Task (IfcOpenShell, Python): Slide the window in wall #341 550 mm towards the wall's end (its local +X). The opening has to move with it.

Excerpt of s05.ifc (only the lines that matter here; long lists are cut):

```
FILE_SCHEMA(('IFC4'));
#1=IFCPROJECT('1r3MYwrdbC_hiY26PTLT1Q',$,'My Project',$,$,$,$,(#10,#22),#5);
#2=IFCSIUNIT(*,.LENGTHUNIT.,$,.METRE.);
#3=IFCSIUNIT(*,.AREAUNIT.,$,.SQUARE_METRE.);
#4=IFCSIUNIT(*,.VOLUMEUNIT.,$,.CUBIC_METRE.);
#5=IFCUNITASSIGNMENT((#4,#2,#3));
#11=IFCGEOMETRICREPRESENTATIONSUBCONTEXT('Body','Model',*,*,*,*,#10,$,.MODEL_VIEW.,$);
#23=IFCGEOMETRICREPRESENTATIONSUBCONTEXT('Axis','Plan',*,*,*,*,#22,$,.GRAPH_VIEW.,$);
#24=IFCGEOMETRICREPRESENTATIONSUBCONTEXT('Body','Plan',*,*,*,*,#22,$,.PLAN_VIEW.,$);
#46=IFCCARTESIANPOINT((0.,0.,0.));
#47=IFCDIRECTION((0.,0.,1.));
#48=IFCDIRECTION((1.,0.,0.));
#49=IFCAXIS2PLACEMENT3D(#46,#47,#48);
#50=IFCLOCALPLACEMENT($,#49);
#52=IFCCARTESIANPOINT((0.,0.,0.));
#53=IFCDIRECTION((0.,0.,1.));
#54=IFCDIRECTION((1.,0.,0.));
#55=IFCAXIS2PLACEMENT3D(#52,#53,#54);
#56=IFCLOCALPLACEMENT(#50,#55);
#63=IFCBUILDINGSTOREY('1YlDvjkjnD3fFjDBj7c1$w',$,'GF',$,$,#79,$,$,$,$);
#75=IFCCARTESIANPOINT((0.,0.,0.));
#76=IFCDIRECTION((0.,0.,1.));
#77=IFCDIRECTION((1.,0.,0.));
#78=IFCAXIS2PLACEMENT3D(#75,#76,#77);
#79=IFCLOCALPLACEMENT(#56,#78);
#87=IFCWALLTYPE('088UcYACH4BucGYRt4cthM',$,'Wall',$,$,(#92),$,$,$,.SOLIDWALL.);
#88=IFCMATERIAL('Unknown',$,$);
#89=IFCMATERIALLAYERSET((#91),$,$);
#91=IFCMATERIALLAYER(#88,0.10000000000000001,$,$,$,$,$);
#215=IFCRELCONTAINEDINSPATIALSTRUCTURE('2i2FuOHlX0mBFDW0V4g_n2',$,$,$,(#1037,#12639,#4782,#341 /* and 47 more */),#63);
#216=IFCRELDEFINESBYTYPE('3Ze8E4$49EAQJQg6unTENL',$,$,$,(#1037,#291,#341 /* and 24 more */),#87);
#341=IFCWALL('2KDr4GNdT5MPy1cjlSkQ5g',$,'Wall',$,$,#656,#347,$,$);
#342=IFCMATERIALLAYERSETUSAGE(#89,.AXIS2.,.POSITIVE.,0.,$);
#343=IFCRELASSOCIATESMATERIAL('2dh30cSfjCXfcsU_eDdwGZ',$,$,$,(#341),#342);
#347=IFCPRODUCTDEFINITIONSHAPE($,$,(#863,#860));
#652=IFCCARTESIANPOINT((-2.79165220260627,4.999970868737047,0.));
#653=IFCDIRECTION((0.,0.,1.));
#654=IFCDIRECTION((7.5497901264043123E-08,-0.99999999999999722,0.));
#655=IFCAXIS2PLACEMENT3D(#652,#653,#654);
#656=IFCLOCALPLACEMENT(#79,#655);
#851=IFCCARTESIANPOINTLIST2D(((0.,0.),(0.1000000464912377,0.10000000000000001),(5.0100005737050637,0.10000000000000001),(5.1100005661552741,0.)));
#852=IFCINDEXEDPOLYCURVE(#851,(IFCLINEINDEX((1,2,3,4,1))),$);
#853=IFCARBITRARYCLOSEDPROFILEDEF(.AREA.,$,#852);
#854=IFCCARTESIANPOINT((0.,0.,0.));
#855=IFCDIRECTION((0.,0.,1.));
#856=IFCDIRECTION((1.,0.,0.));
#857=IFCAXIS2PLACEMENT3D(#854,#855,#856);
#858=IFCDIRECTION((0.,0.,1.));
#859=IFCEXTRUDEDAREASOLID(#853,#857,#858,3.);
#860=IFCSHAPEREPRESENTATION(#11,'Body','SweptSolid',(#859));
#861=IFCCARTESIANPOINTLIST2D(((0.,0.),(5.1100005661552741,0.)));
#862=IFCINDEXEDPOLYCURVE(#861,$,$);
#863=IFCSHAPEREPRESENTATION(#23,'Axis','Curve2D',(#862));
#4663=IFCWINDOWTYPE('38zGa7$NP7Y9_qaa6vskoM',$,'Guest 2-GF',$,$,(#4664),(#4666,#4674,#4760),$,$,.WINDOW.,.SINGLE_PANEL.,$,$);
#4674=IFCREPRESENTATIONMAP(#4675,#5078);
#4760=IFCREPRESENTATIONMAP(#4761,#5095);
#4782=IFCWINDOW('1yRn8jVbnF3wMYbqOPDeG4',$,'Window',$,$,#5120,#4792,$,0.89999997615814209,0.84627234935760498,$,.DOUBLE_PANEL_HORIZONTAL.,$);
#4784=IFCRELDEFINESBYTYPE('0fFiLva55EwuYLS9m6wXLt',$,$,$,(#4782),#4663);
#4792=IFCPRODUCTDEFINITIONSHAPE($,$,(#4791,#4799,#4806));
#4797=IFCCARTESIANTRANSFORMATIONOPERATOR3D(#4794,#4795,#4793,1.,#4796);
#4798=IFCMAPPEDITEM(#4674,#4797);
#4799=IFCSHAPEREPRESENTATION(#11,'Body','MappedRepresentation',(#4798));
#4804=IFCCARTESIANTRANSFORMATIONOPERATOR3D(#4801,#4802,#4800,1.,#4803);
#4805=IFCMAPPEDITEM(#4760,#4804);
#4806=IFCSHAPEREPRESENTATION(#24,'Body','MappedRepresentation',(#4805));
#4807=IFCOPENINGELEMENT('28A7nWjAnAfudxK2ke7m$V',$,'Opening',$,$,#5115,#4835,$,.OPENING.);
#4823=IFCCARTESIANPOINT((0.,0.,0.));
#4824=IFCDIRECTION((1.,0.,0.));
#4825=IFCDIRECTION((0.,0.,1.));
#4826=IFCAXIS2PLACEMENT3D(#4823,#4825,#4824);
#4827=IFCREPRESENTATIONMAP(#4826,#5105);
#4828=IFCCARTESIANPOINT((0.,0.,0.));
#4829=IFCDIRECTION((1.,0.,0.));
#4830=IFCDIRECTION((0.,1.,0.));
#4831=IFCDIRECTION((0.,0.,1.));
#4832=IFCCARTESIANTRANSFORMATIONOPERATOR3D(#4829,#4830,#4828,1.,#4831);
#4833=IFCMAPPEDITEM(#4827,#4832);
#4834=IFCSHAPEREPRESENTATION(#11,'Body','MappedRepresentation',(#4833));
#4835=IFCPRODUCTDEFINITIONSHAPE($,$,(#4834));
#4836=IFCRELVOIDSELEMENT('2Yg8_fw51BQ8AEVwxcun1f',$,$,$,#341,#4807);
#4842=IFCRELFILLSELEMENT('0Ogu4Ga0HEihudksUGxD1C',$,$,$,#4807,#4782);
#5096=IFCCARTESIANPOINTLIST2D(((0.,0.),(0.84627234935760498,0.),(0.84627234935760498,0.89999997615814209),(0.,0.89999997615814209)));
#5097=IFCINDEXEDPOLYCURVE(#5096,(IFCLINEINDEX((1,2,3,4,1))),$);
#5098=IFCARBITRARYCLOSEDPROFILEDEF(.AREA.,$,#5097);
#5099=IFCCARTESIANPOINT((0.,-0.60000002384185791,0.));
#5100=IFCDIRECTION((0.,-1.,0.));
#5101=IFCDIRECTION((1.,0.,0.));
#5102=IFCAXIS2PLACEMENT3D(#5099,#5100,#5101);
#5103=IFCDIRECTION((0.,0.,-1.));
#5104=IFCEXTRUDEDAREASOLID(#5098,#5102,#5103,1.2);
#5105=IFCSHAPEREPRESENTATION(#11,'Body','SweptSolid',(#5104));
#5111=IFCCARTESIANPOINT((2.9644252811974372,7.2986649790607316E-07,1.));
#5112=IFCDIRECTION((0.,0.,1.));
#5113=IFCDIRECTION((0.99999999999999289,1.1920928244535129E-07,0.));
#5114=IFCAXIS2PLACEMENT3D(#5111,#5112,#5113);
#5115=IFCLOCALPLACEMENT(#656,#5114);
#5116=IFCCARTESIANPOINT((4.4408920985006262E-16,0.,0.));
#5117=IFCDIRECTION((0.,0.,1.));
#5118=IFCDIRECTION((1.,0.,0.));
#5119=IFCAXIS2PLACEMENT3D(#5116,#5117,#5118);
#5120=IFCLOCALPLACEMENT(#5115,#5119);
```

```python
import ifcopenshell
import ifcopenshell.api.geometry
import ifcopenshell.util.placement

model = ifcopenshell.open("s05.ifc")

window = model.by_id(4782)
opening = window.FillsVoids[0].RelatingOpeningElement
wall = opening.VoidsElements[0].RelatingBuildingElement

wall_matrix = ifcopenshell.util.placement.get_local_placement(wall.ObjectPlacement)
shift = wall_matrix[:3, 0] * 0.55
before = ifcopenshell.util.placement.get_local_placement(window.ObjectPlacement)[:3, 3].copy()

# The window is placed relative to its opening, so it follows when the opening moves.
matrix = ifcopenshell.util.placement.get_local_placement(opening.ObjectPlacement)
matrix[:3, 3] += shift
ifcopenshell.api.geometry.edit_object_placement(
    model, product=opening, matrix=matrix, is_si=False, should_transform_children=True
)

after = ifcopenshell.util.placement.get_local_placement(window.ObjectPlacement)[:3, 3]
print("window moved by", (after - before).round(3) + 0.0)

model.write("s05_updated.ifc")
```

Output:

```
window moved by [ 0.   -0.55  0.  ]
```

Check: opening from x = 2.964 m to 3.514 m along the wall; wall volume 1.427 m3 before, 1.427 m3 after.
